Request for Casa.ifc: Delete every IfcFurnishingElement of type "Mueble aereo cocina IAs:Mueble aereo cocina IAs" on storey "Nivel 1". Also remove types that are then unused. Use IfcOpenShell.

First a look at what the model holds.

```python
import ifcopenshell
import ifcopenshell.util.element

model = ifcopenshell.open("Casa.ifc")
print(model.schema)
storey = next(s for s in model.by_type("IfcBuildingStorey") if s.Name == "Nivel 1")
furniture = [e for e in ifcopenshell.util.element.get_decomposition(storey) if e.is_a("IfcFurnishingElement")]
seen = {}
for e in furniture:
    element_type = ifcopenshell.util.element.get_type(e)
    name = element_type.Name if element_type not in (None, e) else None
    seen[name] = seen.get(name, 0) + 1
for name, count in sorted(seen.items(), key=str):
    print(count, "x", name)
```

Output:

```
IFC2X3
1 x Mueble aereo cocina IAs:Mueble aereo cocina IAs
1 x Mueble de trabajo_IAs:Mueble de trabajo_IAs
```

```python
import ifcopenshell
import ifcopenshell.api.root
import ifcopenshell.util.element

model = ifcopenshell.open("Casa.ifc")

storey = next(s for s in model.by_type("IfcBuildingStorey") if s.Name == "Nivel 1")
furniture = [e for e in ifcopenshell.util.element.get_decomposition(storey) if e.is_a("IfcFurnishingElement")]
targets = [e for e in furniture if (t := ifcopenshell.util.element.get_type(e)) not in (None, e) and t.Name == "Mueble aereo cocina IAs:Mueble aereo cocina IAs"]
types = {ifcopenshell.util.element.get_type(e) for e in targets} - {None, *targets}

for e in targets:
    ifcopenshell.api.root.remove_product(model, product=e)
print(len(targets), "removed")

unused = [t for t in types if not ifcopenshell.util.element.get_types(t)]
for t in unused:
    ifcopenshell.api.root.remove_product(model, product=t)
print(len(unused), "unused types removed")

model.write("Casa_edited.ifc")
```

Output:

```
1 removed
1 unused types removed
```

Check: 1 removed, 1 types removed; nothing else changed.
